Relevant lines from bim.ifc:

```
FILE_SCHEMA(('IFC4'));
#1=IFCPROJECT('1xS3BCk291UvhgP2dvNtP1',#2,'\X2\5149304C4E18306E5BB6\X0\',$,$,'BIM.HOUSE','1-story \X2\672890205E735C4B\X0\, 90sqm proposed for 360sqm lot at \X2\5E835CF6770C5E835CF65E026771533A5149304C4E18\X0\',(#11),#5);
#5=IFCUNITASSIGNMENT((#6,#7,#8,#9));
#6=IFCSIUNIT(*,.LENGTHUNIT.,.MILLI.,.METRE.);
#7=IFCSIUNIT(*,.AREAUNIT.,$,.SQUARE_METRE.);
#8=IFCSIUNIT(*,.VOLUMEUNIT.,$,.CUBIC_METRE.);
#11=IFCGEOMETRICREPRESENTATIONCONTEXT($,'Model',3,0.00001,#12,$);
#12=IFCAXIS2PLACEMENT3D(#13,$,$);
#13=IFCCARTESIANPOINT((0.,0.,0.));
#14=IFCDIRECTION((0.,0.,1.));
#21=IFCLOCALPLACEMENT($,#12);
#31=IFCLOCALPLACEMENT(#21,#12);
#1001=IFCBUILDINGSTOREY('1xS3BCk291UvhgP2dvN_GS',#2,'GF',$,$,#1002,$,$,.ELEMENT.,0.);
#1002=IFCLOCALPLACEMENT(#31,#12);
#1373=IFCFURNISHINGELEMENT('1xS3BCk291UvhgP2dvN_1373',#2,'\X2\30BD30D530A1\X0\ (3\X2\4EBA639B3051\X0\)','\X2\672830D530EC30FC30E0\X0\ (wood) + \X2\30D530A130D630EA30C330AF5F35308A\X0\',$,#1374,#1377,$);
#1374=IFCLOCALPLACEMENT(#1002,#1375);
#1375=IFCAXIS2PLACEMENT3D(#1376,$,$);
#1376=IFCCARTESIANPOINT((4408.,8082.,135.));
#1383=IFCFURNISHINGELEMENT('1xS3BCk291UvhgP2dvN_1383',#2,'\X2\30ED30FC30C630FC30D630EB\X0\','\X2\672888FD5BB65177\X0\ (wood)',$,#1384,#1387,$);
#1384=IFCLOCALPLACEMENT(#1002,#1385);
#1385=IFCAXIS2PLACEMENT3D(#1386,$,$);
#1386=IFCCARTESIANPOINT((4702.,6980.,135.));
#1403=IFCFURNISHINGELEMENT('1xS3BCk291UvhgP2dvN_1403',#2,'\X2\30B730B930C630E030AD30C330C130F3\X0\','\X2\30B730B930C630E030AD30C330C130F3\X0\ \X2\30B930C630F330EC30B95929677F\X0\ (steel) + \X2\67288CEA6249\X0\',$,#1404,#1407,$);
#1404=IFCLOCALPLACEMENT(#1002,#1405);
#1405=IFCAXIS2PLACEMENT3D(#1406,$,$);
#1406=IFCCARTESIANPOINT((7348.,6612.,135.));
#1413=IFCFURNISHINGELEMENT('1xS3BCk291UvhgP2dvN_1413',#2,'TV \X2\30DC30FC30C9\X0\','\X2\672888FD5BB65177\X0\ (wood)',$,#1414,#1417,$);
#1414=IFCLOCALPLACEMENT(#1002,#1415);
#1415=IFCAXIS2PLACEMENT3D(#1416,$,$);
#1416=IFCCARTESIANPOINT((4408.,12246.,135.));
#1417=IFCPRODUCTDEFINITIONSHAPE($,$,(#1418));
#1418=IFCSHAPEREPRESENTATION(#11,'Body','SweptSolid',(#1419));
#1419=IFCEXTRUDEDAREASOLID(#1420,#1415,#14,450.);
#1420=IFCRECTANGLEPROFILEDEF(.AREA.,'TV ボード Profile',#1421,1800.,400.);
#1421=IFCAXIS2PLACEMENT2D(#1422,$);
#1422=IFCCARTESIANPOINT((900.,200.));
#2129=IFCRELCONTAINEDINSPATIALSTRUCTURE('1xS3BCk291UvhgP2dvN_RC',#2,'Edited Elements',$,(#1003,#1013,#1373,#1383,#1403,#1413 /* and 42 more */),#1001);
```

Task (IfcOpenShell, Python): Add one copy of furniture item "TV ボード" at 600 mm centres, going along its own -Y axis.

```python
import ifcopenshell
import ifcopenshell.api.geometry
import ifcopenshell.api.root
import ifcopenshell.util.element
import ifcopenshell.util.placement

model = ifcopenshell.open("bim.ifc")


def reuse_history(source, copy):
    """copy_class also copies each property set's owner history, people and application; keep the originals."""
    for rel in copy.IsDefinedBy:
        if rel.is_a("IfcRelDefinesByProperties") and (history := rel.RelatingPropertyDefinition.OwnerHistory):
            rel.RelatingPropertyDefinition.OwnerHistory = source.OwnerHistory
            ifcopenshell.util.element.remove_deep2(model, history)


source = model.by_guid("1xS3BCk291UvhgP2dvN_1413")
base = ifcopenshell.util.placement.get_local_placement(source.ObjectPlacement)
step = -base[:3, 1] * 600.0

for i in range(1, 2):
    copy = ifcopenshell.api.root.copy_class(model, product=source)
    copy.Representation = ifcopenshell.util.element.copy_deep(
        model, source.Representation, exclude=["IfcGeometricRepresentationContext", "IfcRepresentationMap"]
    )
    reuse_history(source, copy)
    matrix = base.copy()
    matrix[:3, 3] += i * step
    print("added at", matrix[:3, 3].round(3) + 0.0)
    ifcopenshell.api.geometry.edit_object_placement(model, product=copy, matrix=matrix, is_si=False)

model.write("bim-out.ifc")
```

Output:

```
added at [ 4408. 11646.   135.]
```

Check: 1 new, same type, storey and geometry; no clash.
